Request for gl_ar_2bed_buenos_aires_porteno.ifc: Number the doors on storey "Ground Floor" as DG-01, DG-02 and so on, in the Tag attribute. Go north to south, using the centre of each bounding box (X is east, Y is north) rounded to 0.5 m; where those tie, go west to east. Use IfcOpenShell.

First a look at what the model holds.

```python
import ifcopenshell
import ifcopenshell.util.element
import ifcopenshell.util.placement

model = ifcopenshell.open("gl_ar_2bed_buenos_aires_porteno.ifc")
print(model.schema)
storey = next(s for s in model.by_type("IfcBuildingStorey") if s.Name == "Ground Floor")
doors = [e for e in ifcopenshell.util.element.get_decomposition(storey) if e.is_a("IfcDoor")]
for e in sorted(doors, key=lambda e: e.id()):
    origin = ifcopenshell.util.placement.get_local_placement(e.ObjectPlacement)[:3, 3]
    print(e.id(), e.Tag, e.Name, origin.round(2) + 0.0, sep=" | ")
```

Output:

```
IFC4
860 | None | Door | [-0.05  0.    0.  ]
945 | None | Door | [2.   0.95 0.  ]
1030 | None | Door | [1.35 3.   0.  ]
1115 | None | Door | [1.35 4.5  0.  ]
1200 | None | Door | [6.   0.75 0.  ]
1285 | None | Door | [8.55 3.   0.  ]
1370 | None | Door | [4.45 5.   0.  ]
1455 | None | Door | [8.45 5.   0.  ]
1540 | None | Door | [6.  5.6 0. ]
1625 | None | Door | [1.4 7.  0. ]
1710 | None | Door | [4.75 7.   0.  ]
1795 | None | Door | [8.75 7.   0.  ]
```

```python
import ifcopenshell
import ifcopenshell.geom
import ifcopenshell.util.element
import ifcopenshell.util.shape

model = ifcopenshell.open("gl_ar_2bed_buenos_aires_porteno.ifc")
settings = ifcopenshell.geom.settings()
settings.set("use-world-coords", True)


def centre(element):
    shape = ifcopenshell.geom.create_shape(settings, element)
    return ifcopenshell.util.shape.get_bbox_centroid(shape.geometry)


storey = next(s for s in model.by_type("IfcBuildingStorey") if s.Name == "Ground Floor")
doors = [e for e in ifcopenshell.util.element.get_decomposition(storey) if e.is_a("IfcDoor")]

# Insertion points can sit at a corner or the storey origin, so sort by the geometry (in metres).
centres = {e: centre(e) for e in doors}
doors.sort(key=lambda e: (-round(centres[e][1] / 0.5), centres[e][0]))

for i, e in enumerate(doors, start=1):
    number = f"DG-{i:02d}"
    e.Tag = number
    print(e.id(), number)

model.write("gl_ar_2bed_buenos_aires_porteno_edited.ifc")
```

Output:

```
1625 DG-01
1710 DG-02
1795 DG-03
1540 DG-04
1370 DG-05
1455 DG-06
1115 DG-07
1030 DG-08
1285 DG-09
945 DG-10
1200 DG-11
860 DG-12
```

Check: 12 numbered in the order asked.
